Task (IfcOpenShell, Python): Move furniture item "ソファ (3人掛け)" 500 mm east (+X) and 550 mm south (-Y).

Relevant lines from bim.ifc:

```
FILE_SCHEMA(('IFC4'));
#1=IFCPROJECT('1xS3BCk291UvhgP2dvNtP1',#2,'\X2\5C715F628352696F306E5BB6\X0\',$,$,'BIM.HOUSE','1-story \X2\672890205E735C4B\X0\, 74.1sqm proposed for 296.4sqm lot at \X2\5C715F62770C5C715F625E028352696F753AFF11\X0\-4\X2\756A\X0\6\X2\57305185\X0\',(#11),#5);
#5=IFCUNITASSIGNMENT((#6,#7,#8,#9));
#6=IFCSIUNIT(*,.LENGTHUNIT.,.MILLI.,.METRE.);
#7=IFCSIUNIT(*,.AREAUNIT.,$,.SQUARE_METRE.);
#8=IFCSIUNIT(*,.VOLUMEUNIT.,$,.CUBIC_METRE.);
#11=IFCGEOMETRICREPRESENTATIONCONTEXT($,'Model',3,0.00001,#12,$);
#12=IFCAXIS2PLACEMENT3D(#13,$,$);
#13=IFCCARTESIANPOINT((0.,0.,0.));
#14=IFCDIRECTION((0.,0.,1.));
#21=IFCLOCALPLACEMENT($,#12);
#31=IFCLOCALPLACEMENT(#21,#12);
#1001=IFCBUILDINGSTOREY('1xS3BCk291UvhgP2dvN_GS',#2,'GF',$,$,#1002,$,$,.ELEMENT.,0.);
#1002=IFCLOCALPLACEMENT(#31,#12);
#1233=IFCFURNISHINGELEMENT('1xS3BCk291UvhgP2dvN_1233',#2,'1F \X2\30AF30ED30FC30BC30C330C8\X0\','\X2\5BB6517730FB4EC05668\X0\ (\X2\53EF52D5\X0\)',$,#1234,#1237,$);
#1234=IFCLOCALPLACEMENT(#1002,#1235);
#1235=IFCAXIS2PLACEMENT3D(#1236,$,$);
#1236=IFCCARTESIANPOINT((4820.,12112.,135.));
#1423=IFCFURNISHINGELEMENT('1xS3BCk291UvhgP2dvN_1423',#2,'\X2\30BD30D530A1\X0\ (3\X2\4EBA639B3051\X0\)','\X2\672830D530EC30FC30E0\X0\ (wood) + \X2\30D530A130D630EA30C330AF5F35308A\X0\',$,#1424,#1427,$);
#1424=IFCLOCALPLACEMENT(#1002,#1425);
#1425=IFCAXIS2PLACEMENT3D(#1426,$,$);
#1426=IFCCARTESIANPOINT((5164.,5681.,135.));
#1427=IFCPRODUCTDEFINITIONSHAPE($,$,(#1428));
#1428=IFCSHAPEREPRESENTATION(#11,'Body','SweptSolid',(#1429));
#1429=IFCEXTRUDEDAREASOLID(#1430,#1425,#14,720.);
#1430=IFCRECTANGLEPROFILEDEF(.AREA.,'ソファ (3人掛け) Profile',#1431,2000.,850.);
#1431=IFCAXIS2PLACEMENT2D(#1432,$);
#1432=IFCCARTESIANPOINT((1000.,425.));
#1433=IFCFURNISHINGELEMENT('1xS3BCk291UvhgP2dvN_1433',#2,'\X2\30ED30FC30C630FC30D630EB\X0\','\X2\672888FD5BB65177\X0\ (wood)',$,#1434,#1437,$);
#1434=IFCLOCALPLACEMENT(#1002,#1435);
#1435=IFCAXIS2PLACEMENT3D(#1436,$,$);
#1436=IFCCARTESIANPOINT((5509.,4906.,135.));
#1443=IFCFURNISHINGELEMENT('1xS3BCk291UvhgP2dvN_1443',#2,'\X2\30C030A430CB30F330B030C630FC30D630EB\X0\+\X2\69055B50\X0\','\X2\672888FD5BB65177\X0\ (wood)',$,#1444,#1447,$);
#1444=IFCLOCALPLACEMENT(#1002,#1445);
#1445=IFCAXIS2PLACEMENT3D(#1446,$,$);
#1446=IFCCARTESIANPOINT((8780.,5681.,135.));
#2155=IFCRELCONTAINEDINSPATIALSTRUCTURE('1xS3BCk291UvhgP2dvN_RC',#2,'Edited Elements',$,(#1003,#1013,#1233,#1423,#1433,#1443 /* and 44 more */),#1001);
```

```python
import ifcopenshell
import ifcopenshell.api.geometry
import ifcopenshell.util.placement

model = ifcopenshell.open("bim.ifc")

item = model.by_guid("1xS3BCk291UvhgP2dvN_1423")
matrix = ifcopenshell.util.placement.get_local_placement(item.ObjectPlacement)
matrix[0, 3] += 500.0
matrix[1, 3] -= 550.0
ifcopenshell.api.geometry.edit_object_placement(model, product=item, matrix=matrix, is_si=False)

print(ifcopenshell.util.placement.get_local_placement(item.ObjectPlacement).round(3) + 0.0)

model.write("bim_v2.ifc")
```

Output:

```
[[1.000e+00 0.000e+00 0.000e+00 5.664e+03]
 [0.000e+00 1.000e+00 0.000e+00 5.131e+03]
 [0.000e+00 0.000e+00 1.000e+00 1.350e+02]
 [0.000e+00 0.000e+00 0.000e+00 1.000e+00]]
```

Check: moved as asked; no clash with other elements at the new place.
